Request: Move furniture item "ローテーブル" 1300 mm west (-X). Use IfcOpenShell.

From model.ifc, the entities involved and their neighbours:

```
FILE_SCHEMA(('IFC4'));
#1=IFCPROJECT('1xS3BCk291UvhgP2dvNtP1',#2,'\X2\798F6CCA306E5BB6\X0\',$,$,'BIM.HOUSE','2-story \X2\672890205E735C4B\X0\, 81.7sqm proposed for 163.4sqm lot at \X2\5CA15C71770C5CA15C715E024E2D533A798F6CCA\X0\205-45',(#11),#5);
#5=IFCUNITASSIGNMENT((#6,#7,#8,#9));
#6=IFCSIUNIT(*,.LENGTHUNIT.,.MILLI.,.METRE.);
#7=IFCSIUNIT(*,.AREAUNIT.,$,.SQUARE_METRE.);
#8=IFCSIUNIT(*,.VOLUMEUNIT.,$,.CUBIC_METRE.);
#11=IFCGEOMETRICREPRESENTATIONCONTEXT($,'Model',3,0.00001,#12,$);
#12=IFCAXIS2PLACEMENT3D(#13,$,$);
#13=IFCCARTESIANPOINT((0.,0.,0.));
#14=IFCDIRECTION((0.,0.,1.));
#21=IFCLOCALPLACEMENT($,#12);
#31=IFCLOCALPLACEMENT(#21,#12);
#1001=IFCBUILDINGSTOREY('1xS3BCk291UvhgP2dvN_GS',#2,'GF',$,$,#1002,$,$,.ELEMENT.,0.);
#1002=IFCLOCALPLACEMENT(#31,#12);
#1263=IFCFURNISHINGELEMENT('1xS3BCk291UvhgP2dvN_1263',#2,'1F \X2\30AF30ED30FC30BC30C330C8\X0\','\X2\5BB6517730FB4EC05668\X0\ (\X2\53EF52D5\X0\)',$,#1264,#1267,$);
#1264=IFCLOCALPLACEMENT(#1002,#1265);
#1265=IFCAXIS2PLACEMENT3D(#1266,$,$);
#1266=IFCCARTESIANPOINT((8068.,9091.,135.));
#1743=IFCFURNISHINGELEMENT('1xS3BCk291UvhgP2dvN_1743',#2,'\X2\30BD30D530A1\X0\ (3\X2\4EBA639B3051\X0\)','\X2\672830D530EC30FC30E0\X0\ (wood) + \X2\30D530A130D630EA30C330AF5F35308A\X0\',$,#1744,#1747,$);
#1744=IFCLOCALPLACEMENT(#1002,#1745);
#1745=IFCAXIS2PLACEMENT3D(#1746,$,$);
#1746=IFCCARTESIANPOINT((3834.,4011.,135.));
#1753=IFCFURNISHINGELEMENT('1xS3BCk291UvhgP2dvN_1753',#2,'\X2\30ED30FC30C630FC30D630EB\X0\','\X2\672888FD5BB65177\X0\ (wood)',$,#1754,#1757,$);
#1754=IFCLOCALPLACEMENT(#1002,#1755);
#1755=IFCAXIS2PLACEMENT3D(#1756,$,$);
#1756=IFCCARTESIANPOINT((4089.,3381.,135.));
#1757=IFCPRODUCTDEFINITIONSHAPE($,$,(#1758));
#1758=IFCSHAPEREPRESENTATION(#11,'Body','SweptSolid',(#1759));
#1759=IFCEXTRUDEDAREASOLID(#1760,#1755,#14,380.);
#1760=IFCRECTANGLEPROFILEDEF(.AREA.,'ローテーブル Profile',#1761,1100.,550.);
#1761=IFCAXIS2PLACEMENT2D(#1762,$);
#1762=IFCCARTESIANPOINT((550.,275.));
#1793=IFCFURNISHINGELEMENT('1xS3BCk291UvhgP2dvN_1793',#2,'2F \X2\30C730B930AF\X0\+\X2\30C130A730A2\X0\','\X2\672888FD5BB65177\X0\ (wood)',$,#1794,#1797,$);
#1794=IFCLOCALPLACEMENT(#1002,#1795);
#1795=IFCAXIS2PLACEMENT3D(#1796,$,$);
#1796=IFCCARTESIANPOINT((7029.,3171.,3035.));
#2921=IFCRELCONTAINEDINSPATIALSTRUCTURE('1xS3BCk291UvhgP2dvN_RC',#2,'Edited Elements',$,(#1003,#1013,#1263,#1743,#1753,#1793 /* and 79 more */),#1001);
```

```python
import ifcopenshell
import ifcopenshell.api.geometry
import ifcopenshell.util.placement

model = ifcopenshell.open("model.ifc")

item = model.by_id(1753)
matrix = ifcopenshell.util.placement.get_local_placement(item.ObjectPlacement)
matrix[0, 3] -= 1300.0
ifcopenshell.api.geometry.edit_object_placement(model, product=item, matrix=matrix, is_si=False)

print(ifcopenshell.util.placement.get_local_placement(item.ObjectPlacement).round(3) + 0.0)

model.write("model_updated.ifc")
```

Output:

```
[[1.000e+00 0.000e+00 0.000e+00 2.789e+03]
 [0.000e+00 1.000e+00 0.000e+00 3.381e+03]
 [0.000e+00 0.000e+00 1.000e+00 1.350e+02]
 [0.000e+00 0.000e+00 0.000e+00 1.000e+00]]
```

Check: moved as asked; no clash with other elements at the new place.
